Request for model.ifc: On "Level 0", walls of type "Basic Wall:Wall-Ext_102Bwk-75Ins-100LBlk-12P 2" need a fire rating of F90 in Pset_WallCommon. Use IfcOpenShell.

First a look at what the model holds.

```python
import ifcopenshell
import ifcopenshell.util.element

model = ifcopenshell.open("model.ifc")
print(model.schema)
storey = next(s for s in model.by_type("IfcBuildingStorey") if s.Name == "Level 0")
walls = [e for e in ifcopenshell.util.element.get_decomposition(storey) if e.is_a("IfcWall")]
seen = {}
for e in walls:
    element_type = ifcopenshell.util.element.get_type(e)
    key = (element_type.Name if element_type != e and element_type else None, ifcopenshell.util.element.get_pset(e, "Pset_WallCommon", "FireRating"))
    seen[key] = seen.get(key, 0) + 1
for (name, value), count in sorted(seen.items(), key=str):
    print(count, "x", name, "|", value)
```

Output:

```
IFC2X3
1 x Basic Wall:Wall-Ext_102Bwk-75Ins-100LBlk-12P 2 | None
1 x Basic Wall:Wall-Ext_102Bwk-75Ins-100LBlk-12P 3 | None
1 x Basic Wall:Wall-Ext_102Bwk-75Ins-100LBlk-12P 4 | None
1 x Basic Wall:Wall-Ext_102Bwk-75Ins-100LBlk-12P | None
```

```python
import ifcopenshell
import ifcopenshell.api.pset
import ifcopenshell.util.element

model = ifcopenshell.open("model.ifc")

storey = next(s for s in model.by_type("IfcBuildingStorey") if s.Name == "Level 0")
walls = [e for e in ifcopenshell.util.element.get_decomposition(storey) if e.is_a("IfcWall")]

count = 0
for e in walls:
    element_type = ifcopenshell.util.element.get_type(e)
    if element_type in (None, e) or element_type.Name != "Basic Wall:Wall-Ext_102Bwk-75Ins-100LBlk-12P 2":
        continue
    # add_pset returns the element's existing set when there is one.
    pset = ifcopenshell.api.pset.add_pset(model, product=e, name="Pset_WallCommon")
    ifcopenshell.api.pset.edit_pset(model, pset=pset, properties={"FireRating": "F90"})
    count += 1

print(count, "walls updated")

model.write("model-out.ifc")
```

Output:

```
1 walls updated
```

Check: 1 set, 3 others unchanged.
